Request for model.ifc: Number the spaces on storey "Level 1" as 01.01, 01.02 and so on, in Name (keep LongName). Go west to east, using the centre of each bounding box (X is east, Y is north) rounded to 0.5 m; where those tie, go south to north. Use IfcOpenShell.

First a look at what the model holds.

```python
import ifcopenshell
import ifcopenshell.util.element
import ifcopenshell.util.placement

model = ifcopenshell.open("model.ifc")
print(model.schema)
storey = next(s for s in model.by_type("IfcBuildingStorey") if s.Name == "Level 1")
spaces = [e for e in ifcopenshell.util.element.get_decomposition(storey) if e.is_a("IfcSpace")]
for e in sorted(spaces, key=lambda e: e.id()):
    origin = ifcopenshell.util.placement.get_local_placement(e.ObjectPlacement)[:3, 3]
    print(e.id(), e.Name, e.LongName, origin.round(2) + 0.0, sep=" | ")
```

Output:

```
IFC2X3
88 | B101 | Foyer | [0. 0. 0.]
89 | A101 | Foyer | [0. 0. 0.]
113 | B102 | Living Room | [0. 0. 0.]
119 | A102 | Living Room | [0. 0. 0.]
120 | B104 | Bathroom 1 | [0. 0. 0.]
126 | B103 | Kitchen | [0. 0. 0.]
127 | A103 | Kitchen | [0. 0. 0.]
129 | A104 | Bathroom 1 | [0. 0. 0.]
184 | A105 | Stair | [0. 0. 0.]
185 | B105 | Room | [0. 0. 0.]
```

```python
import ifcopenshell
import ifcopenshell.geom
import ifcopenshell.util.element
import ifcopenshell.util.shape

model = ifcopenshell.open("model.ifc")
settings = ifcopenshell.geom.settings()
settings.set("use-world-coords", True)


def centre(element):
    shape = ifcopenshell.geom.create_shape(settings, element)
    return ifcopenshell.util.shape.get_bbox_centroid(shape.geometry)


storey = next(s for s in model.by_type("IfcBuildingStorey") if s.Name == "Level 1")
spaces = [e for e in ifcopenshell.util.element.get_decomposition(storey) if e.is_a("IfcSpace")]

# Insertion points can sit at a corner or the storey origin, so sort by the geometry (in metres).
centres = {e: centre(e) for e in spaces}
spaces.sort(key=lambda e: (round(centres[e][0] / 0.5), centres[e][1]))

for i, e in enumerate(spaces, start=1):
    number = f"01.{i:02d}"
    e.Name = number
    print(e.id(), number)

model.write("model_edited.ifc")
```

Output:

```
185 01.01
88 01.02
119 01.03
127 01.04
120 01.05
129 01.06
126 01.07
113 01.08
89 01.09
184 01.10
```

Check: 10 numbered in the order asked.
